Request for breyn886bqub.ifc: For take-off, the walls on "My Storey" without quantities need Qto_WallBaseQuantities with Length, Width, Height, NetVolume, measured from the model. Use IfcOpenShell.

First a look at what the model holds.

```python
import ifcopenshell
import ifcopenshell.util.element
import ifcopenshell.util.unit

model = ifcopenshell.open("breyn886bqub.ifc")
print(model.schema)
for unit_type in ("LENGTHUNIT", "AREAUNIT", "VOLUMEUNIT"):
    print(unit_type, ifcopenshell.util.unit.calculate_unit_scale(model, unit_type))
storey = next(s for s in model.by_type("IfcBuildingStorey") if s.Name == "My Storey")
walls = [e for e in ifcopenshell.util.element.get_decomposition(storey) if e.is_a("IfcWall")]
for e in sorted(walls, key=lambda e: e.id()):
    print(e.id(), e.is_a(), e.Name, list(ifcopenshell.util.element.get_psets(e, qtos_only=True)), sep=" | ")
```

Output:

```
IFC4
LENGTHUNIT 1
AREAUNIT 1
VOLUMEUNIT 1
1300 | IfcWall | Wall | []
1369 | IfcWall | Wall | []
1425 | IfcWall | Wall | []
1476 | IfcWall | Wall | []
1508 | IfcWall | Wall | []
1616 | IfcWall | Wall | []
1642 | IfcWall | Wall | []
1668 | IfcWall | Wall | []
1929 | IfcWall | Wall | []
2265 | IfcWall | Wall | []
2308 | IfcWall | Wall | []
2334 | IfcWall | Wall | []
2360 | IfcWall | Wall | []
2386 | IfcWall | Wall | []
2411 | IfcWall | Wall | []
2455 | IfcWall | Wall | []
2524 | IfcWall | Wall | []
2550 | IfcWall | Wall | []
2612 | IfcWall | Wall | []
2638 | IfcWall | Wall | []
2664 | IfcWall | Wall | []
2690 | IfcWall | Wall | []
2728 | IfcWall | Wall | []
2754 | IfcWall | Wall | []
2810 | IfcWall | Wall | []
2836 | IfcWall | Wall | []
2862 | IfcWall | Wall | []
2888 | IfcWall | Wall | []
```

```python
import ifcopenshell
import ifcopenshell.api.pset
import ifcopenshell.geom
import ifcopenshell.util.element
import ifcopenshell.util.shape
import ifcopenshell.util.unit

model = ifcopenshell.open("breyn886bqub.ifc")
unit_scale = ifcopenshell.util.unit.calculate_unit_scale(model)
volume_scale = ifcopenshell.util.unit.calculate_unit_scale(model, "VOLUMEUNIT")
settings = ifcopenshell.geom.settings()

storey = next(s for s in model.by_type("IfcBuildingStorey") if s.Name == "My Storey")
walls = [e for e in ifcopenshell.util.element.get_decomposition(storey) if e.is_a("IfcWall")]

for e in sorted(walls, key=lambda e: e.id()):
    if ifcopenshell.util.element.get_psets(e, qtos_only=True, should_inherit=False):
        continue
    # Geometry comes back in metres, in the element's own axes.
    shape = ifcopenshell.geom.create_shape(settings, e)
    values = {
        "Length": ifcopenshell.util.shape.get_x(shape.geometry) / unit_scale,
        "Width": ifcopenshell.util.shape.get_y(shape.geometry) / unit_scale,
        "Height": ifcopenshell.util.shape.get_z(shape.geometry) / unit_scale,
        "NetVolume": ifcopenshell.util.shape.get_volume(shape.geometry) / volume_scale,
    }
    qto = ifcopenshell.api.pset.add_qto(model, product=e, name="Qto_WallBaseQuantities")
    ifcopenshell.api.pset.edit_qto(model, qto=qto, properties=values)
    print(e.id(), {k: round(v, 3) for k, v in values.items()})

model.write("breyn886bqub_updated.ifc")
```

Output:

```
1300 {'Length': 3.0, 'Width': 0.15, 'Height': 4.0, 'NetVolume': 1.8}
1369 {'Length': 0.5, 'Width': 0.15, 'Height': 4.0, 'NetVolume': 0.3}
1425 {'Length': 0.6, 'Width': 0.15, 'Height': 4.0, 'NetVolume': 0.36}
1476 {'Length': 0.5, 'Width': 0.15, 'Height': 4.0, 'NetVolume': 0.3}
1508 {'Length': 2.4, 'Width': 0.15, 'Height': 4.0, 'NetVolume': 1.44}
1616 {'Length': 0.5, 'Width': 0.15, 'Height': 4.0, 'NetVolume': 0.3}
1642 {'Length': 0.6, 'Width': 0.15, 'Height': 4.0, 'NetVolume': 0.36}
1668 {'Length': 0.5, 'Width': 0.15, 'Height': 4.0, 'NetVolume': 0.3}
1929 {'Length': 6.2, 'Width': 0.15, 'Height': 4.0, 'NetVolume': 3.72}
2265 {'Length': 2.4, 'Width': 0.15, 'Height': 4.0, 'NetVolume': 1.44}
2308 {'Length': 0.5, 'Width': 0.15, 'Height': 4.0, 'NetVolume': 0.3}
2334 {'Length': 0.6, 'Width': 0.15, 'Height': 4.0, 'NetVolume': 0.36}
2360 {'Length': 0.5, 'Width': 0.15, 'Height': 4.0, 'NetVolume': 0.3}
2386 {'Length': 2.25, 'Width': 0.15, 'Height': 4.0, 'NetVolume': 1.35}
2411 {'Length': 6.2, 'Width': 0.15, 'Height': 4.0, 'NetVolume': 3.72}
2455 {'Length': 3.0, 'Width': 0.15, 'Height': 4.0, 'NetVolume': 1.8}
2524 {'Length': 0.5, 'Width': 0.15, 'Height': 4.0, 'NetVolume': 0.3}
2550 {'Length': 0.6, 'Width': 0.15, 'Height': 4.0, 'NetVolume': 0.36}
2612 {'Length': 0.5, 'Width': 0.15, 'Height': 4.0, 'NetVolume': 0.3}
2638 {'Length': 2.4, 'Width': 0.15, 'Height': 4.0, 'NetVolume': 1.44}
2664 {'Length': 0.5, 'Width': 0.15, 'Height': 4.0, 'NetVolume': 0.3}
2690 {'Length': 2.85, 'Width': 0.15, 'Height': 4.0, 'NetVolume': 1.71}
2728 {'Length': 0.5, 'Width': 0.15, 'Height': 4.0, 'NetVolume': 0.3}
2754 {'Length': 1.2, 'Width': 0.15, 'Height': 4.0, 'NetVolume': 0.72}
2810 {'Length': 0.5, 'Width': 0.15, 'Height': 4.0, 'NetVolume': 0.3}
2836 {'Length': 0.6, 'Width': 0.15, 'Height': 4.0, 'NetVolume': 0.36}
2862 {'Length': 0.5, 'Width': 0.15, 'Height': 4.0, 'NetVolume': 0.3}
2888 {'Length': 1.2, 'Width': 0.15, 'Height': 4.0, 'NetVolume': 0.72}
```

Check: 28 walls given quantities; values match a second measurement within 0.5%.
